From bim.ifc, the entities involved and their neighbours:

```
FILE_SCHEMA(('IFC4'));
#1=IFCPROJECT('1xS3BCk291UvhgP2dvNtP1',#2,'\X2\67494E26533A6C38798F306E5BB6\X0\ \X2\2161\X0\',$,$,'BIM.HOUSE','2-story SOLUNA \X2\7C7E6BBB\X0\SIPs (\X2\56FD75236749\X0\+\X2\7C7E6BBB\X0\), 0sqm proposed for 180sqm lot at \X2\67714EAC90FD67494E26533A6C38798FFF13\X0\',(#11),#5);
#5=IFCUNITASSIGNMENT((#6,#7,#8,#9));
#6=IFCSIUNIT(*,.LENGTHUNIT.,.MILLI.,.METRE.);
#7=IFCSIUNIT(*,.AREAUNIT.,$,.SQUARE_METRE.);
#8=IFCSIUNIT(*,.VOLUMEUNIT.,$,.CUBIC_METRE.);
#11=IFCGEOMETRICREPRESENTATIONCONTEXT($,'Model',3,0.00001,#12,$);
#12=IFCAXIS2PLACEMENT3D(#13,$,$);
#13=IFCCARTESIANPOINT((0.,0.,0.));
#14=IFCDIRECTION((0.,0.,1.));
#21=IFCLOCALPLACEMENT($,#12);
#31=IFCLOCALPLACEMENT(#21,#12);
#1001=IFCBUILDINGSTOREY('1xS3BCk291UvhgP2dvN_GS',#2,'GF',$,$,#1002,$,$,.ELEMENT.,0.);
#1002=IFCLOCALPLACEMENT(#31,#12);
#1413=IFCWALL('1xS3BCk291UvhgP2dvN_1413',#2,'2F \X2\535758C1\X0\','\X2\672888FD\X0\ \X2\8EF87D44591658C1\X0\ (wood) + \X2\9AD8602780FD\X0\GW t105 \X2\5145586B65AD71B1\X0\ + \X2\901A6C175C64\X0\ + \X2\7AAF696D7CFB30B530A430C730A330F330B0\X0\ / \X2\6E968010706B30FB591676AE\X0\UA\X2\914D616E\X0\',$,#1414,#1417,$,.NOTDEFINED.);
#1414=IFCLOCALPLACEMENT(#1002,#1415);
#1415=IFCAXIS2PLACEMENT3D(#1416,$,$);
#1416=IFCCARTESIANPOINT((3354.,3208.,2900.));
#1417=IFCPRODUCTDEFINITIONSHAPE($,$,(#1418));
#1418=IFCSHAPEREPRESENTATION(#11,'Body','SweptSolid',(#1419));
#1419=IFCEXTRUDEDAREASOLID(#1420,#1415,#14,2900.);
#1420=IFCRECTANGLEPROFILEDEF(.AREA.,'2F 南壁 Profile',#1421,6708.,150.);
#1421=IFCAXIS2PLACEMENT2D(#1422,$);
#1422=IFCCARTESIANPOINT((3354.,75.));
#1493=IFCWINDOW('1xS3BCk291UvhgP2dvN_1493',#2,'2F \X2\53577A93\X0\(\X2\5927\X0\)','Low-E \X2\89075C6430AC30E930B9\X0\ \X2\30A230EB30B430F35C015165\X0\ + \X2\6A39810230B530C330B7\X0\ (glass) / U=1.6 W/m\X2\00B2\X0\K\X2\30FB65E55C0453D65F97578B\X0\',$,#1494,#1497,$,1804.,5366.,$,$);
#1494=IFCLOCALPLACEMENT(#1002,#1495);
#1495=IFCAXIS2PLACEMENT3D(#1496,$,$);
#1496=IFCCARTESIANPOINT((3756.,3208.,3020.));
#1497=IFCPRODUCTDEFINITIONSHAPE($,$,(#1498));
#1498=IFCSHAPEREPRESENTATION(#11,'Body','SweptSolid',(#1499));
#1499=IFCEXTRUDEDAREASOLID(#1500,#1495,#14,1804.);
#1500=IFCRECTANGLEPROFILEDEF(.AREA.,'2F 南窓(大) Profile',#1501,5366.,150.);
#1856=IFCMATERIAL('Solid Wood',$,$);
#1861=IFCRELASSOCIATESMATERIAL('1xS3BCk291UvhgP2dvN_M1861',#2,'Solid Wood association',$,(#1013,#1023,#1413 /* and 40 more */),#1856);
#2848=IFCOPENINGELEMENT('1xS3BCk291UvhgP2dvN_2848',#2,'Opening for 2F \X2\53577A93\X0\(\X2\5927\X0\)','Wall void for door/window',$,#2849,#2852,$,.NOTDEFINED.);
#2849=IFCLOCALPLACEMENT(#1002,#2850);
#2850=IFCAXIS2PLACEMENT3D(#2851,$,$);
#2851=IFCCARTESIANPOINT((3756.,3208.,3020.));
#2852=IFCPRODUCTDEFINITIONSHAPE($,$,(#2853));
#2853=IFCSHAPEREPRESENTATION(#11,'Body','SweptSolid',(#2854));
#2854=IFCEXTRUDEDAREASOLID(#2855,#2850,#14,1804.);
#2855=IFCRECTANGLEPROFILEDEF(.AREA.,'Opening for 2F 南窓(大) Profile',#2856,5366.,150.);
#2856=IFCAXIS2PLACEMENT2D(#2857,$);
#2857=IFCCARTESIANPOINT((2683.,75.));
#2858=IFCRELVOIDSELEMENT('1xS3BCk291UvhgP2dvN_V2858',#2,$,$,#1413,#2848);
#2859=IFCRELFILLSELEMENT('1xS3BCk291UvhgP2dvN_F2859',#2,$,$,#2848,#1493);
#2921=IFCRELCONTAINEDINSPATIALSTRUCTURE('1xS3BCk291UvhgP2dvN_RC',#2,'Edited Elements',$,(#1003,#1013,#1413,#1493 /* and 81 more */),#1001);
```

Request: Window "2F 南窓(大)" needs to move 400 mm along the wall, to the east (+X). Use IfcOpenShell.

```python
import ifcopenshell
import ifcopenshell.api.geometry
import ifcopenshell.util.placement
import ifcopenshell.util.unit

model = ifcopenshell.open("bim.ifc")
unit_scale = ifcopenshell.util.unit.calculate_unit_scale(model)

window = model.by_id(1493)
opening = window.FillsVoids[0].RelatingOpeningElement
wall = opening.VoidsElements[0].RelatingBuildingElement

wall_matrix = ifcopenshell.util.placement.get_local_placement(wall.ObjectPlacement)
shift = wall_matrix[:3, 0] * 0.4 / unit_scale
before = ifcopenshell.util.placement.get_local_placement(window.ObjectPlacement)[:3, 3].copy()

# The window is not placed relative to its opening, so move both.
for product in (opening, window):
    matrix = ifcopenshell.util.placement.get_local_placement(product.ObjectPlacement)
    matrix[:3, 3] += shift
    ifcopenshell.api.geometry.edit_object_placement(model, product=product, matrix=matrix, is_si=False)

after = ifcopenshell.util.placement.get_local_placement(window.ObjectPlacement)[:3, 3]
print("window moved by", (after - before).round(3) + 0.0)

model.write("bim-out.ifc")
```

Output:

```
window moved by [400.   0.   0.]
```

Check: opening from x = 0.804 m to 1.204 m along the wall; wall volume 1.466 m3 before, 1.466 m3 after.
